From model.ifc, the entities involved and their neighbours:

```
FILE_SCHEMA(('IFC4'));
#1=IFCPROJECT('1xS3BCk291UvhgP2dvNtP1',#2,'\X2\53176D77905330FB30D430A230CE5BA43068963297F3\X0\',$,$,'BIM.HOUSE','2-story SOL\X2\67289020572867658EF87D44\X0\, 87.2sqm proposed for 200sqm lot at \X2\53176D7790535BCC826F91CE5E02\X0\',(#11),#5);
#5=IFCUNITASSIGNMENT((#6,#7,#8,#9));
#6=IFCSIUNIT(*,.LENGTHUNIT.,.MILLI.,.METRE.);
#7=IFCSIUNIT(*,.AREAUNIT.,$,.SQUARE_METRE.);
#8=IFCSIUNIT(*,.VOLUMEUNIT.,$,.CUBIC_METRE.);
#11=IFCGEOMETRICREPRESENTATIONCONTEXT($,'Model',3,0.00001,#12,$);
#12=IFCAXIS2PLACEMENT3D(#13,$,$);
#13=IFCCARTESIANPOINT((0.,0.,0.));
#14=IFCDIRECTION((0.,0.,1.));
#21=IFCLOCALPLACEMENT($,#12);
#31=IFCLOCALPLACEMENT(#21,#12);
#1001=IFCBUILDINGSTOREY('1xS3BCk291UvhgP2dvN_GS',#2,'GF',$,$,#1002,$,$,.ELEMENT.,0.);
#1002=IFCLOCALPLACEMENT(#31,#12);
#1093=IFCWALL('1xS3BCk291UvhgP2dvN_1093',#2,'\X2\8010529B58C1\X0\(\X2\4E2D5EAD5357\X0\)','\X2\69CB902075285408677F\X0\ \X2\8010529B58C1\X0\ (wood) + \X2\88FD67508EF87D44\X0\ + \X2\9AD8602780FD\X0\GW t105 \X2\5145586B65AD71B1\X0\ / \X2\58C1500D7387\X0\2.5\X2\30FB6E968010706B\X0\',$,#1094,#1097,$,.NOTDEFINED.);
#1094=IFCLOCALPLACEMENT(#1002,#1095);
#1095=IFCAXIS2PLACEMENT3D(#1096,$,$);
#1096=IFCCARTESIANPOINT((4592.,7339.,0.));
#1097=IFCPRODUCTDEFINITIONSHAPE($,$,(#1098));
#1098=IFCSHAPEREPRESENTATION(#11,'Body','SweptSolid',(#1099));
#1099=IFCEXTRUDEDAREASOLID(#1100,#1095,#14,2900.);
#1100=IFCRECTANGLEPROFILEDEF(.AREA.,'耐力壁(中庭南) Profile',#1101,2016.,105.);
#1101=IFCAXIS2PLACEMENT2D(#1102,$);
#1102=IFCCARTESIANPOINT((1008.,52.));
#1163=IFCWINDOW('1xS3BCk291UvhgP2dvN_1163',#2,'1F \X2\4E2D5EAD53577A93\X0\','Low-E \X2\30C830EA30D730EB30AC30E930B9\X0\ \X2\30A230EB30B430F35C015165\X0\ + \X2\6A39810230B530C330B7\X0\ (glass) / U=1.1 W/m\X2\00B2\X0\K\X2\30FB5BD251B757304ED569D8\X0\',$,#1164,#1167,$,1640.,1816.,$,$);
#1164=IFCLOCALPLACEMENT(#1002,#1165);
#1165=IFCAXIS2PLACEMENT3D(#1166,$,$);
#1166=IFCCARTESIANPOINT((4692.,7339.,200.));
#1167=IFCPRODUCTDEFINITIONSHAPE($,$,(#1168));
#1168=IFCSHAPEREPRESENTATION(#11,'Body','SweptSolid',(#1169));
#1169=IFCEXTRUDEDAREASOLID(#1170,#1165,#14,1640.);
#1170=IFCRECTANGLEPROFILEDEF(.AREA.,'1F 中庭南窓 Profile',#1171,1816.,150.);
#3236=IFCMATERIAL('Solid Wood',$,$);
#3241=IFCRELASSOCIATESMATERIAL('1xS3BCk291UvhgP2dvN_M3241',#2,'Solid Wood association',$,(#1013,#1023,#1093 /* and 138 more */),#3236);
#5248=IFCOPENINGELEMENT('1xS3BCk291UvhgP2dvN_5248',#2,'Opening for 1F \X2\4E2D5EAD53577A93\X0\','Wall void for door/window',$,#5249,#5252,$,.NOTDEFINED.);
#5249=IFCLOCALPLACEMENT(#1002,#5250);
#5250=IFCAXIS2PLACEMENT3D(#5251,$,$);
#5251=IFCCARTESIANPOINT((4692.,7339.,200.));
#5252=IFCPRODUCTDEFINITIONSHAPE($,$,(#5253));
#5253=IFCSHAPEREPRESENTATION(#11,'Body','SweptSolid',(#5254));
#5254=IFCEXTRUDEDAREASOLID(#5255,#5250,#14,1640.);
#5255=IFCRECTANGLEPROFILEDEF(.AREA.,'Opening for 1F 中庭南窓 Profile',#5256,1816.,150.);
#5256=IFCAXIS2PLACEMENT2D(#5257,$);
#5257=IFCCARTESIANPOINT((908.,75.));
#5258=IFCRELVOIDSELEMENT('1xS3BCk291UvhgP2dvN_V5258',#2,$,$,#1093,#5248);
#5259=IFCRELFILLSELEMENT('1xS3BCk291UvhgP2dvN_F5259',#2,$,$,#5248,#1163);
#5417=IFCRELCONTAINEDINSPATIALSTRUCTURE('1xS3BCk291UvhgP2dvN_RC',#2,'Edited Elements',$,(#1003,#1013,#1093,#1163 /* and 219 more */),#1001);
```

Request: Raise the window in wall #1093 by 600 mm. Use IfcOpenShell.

```python
import numpy as np
import ifcopenshell
import ifcopenshell.api.geometry
import ifcopenshell.util.placement
import ifcopenshell.util.unit

model = ifcopenshell.open("model.ifc")
unit_scale = ifcopenshell.util.unit.calculate_unit_scale(model)

window = model.by_guid("1xS3BCk291UvhgP2dvN_1163")
opening = window.FillsVoids[0].RelatingOpeningElement
dz = 0.6 / unit_scale

shift = np.array([0.0, 0.0, dz])
# The window is not placed relative to its opening, so move both.
for product in (opening, window):
    matrix = ifcopenshell.util.placement.get_local_placement(product.ObjectPlacement)
    matrix[:3, 3] += shift
    ifcopenshell.api.geometry.edit_object_placement(model, product=product, matrix=matrix, is_si=False)

print(f"moved by {dz * unit_scale:+.3f} m")

model.write("model_updated.ifc")
```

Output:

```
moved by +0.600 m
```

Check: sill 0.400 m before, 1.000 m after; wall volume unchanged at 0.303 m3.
